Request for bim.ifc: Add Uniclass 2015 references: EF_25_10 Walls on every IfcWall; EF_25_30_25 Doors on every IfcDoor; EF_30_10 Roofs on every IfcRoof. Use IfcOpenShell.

First a look at what the model holds.

```python
import ifcopenshell

model = ifcopenshell.open("bim.ifc")
print(model.schema)
print("classifications:", [c.Name for c in model.by_type("IfcClassification")])
for ifc_class in ("IfcDoor", "IfcRoof", "IfcStair", "IfcWall", "IfcWindow"):
    print(ifc_class, len(model.by_type(ifc_class)))
```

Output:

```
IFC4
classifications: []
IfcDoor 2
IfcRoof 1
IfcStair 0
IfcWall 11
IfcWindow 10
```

```python
import ifcopenshell
import ifcopenshell.api.classification

model = ifcopenshell.open("bim.ifc")

system = ifcopenshell.api.classification.add_classification(model, classification="Uniclass 2015")

codes = {
    "IfcWall": ("EF_25_10", "Walls"),
    "IfcDoor": ("EF_25_30_25", "Doors"),
    "IfcRoof": ("EF_30_10", "Roofs"),
}
for ifc_class, (code, name) in codes.items():
    products = model.by_type(ifc_class)
    ifcopenshell.api.classification.add_reference(
        model, products=products, classification=system, identification=code, name=name
    )
    print(code, len(products))

model.write("bim_edited.ifc")
```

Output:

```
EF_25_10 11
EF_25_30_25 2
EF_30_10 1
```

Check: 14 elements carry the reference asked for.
